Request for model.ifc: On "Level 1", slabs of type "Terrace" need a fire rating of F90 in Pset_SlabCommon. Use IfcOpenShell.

First a look at what the model holds.

```python
import ifcopenshell
import ifcopenshell.util.element

model = ifcopenshell.open("model.ifc")
print(model.schema)
storey = next(s for s in model.by_type("IfcBuildingStorey") if s.Name == "Level 1")
slabs = [e for e in ifcopenshell.util.element.get_decomposition(storey) if e.is_a("IfcSlab")]
seen = {}
for e in slabs:
    element_type = ifcopenshell.util.element.get_type(e)
    key = (element_type.Name if element_type != e and element_type else None, ifcopenshell.util.element.get_pset(e, "Pset_SlabCommon", "FireRating"))
    seen[key] = seen.get(key, 0) + 1
for (name, value), count in sorted(seen.items(), key=str):
    print(count, "x", name, "|", value)
```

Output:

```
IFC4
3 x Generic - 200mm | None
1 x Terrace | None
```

```python
import ifcopenshell
import ifcopenshell.api.pset
import ifcopenshell.util.element

model = ifcopenshell.open("model.ifc")

storey = next(s for s in model.by_type("IfcBuildingStorey") if s.Name == "Level 1")
slabs = [e for e in ifcopenshell.util.element.get_decomposition(storey) if e.is_a("IfcSlab")]

count = 0
for e in slabs:
    element_type = ifcopenshell.util.element.get_type(e)
    if element_type in (None, e) or element_type.Name != "Terrace":
        continue
    # add_pset returns the element's existing set when there is one.
    pset = ifcopenshell.api.pset.add_pset(model, product=e, name="Pset_SlabCommon")
    ifcopenshell.api.pset.edit_pset(model, pset=pset, properties={"FireRating": "F90"})
    count += 1

print(count, "slabs updated")

model.write("model_rev.ifc")
```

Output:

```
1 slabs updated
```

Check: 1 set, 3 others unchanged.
